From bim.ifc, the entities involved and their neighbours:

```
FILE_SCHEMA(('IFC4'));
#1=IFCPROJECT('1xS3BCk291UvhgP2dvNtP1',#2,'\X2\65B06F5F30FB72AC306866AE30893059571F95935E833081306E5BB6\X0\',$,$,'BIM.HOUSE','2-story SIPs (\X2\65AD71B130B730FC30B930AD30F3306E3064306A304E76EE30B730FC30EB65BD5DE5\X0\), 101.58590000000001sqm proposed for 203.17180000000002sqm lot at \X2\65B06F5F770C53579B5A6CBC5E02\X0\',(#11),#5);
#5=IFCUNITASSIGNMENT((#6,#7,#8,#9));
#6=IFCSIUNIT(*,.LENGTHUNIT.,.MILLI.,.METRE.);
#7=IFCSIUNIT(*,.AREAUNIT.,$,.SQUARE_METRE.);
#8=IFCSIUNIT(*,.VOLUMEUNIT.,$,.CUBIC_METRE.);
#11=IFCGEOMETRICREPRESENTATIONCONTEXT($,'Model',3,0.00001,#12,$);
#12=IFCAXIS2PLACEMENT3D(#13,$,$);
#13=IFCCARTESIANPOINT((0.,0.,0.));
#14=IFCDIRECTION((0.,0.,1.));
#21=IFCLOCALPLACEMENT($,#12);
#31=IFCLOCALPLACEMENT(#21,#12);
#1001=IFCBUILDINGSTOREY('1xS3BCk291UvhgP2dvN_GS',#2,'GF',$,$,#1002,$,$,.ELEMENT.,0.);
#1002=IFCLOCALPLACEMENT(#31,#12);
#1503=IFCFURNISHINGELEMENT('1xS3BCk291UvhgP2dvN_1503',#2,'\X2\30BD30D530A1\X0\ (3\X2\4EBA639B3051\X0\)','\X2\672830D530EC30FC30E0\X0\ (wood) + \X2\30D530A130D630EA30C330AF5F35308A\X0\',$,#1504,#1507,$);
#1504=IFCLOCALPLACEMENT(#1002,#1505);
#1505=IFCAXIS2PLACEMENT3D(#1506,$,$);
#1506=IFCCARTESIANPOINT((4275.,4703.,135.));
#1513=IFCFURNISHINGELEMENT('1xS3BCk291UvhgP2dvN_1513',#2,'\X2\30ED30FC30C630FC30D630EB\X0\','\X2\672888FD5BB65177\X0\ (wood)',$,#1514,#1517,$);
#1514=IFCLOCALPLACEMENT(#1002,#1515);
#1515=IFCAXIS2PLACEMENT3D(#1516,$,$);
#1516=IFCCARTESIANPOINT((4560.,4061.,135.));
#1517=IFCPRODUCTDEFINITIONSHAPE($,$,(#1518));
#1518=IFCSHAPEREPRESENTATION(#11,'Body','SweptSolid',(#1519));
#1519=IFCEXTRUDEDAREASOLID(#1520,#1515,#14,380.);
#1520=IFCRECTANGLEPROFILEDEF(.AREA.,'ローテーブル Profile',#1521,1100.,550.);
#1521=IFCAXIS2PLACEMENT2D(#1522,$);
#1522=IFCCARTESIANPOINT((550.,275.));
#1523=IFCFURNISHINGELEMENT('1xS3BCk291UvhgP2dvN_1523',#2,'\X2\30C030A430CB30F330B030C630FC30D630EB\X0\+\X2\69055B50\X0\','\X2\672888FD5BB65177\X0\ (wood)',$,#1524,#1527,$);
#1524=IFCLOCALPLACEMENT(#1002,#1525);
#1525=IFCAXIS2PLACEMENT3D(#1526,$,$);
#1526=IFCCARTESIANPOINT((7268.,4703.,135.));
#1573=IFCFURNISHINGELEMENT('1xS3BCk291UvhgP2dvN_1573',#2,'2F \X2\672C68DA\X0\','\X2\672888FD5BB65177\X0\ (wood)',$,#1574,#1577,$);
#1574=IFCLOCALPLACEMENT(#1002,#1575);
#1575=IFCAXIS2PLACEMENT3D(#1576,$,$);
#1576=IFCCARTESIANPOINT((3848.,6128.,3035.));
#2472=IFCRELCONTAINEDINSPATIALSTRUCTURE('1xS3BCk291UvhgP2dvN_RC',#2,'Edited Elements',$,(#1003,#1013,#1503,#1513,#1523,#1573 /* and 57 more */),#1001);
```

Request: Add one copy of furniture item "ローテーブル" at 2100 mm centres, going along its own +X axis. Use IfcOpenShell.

```python
import ifcopenshell
import ifcopenshell.api.geometry
import ifcopenshell.api.root
import ifcopenshell.util.element
import ifcopenshell.util.placement

model = ifcopenshell.open("bim.ifc")


def reuse_history(source, copy):
    """copy_class also copies each property set's owner history, people and application; keep the originals."""
    for rel in copy.IsDefinedBy:
        if rel.is_a("IfcRelDefinesByProperties") and (history := rel.RelatingPropertyDefinition.OwnerHistory):
            rel.RelatingPropertyDefinition.OwnerHistory = source.OwnerHistory
            ifcopenshell.util.element.remove_deep2(model, history)


source = model.by_guid("1xS3BCk291UvhgP2dvN_1513")
base = ifcopenshell.util.placement.get_local_placement(source.ObjectPlacement)
step = base[:3, 0] * 2100.0

for i in range(1, 2):
    copy = ifcopenshell.api.root.copy_class(model, product=source)
    copy.Representation = ifcopenshell.util.element.copy_deep(
        model, source.Representation, exclude=["IfcGeometricRepresentationContext", "IfcRepresentationMap"]
    )
    reuse_history(source, copy)
    matrix = base.copy()
    matrix[:3, 3] += i * step
    print("added at", matrix[:3, 3].round(3) + 0.0)
    ifcopenshell.api.geometry.edit_object_placement(model, product=copy, matrix=matrix, is_si=False)

model.write("bim-out.ifc")
```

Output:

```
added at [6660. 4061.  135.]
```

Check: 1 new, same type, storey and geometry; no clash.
